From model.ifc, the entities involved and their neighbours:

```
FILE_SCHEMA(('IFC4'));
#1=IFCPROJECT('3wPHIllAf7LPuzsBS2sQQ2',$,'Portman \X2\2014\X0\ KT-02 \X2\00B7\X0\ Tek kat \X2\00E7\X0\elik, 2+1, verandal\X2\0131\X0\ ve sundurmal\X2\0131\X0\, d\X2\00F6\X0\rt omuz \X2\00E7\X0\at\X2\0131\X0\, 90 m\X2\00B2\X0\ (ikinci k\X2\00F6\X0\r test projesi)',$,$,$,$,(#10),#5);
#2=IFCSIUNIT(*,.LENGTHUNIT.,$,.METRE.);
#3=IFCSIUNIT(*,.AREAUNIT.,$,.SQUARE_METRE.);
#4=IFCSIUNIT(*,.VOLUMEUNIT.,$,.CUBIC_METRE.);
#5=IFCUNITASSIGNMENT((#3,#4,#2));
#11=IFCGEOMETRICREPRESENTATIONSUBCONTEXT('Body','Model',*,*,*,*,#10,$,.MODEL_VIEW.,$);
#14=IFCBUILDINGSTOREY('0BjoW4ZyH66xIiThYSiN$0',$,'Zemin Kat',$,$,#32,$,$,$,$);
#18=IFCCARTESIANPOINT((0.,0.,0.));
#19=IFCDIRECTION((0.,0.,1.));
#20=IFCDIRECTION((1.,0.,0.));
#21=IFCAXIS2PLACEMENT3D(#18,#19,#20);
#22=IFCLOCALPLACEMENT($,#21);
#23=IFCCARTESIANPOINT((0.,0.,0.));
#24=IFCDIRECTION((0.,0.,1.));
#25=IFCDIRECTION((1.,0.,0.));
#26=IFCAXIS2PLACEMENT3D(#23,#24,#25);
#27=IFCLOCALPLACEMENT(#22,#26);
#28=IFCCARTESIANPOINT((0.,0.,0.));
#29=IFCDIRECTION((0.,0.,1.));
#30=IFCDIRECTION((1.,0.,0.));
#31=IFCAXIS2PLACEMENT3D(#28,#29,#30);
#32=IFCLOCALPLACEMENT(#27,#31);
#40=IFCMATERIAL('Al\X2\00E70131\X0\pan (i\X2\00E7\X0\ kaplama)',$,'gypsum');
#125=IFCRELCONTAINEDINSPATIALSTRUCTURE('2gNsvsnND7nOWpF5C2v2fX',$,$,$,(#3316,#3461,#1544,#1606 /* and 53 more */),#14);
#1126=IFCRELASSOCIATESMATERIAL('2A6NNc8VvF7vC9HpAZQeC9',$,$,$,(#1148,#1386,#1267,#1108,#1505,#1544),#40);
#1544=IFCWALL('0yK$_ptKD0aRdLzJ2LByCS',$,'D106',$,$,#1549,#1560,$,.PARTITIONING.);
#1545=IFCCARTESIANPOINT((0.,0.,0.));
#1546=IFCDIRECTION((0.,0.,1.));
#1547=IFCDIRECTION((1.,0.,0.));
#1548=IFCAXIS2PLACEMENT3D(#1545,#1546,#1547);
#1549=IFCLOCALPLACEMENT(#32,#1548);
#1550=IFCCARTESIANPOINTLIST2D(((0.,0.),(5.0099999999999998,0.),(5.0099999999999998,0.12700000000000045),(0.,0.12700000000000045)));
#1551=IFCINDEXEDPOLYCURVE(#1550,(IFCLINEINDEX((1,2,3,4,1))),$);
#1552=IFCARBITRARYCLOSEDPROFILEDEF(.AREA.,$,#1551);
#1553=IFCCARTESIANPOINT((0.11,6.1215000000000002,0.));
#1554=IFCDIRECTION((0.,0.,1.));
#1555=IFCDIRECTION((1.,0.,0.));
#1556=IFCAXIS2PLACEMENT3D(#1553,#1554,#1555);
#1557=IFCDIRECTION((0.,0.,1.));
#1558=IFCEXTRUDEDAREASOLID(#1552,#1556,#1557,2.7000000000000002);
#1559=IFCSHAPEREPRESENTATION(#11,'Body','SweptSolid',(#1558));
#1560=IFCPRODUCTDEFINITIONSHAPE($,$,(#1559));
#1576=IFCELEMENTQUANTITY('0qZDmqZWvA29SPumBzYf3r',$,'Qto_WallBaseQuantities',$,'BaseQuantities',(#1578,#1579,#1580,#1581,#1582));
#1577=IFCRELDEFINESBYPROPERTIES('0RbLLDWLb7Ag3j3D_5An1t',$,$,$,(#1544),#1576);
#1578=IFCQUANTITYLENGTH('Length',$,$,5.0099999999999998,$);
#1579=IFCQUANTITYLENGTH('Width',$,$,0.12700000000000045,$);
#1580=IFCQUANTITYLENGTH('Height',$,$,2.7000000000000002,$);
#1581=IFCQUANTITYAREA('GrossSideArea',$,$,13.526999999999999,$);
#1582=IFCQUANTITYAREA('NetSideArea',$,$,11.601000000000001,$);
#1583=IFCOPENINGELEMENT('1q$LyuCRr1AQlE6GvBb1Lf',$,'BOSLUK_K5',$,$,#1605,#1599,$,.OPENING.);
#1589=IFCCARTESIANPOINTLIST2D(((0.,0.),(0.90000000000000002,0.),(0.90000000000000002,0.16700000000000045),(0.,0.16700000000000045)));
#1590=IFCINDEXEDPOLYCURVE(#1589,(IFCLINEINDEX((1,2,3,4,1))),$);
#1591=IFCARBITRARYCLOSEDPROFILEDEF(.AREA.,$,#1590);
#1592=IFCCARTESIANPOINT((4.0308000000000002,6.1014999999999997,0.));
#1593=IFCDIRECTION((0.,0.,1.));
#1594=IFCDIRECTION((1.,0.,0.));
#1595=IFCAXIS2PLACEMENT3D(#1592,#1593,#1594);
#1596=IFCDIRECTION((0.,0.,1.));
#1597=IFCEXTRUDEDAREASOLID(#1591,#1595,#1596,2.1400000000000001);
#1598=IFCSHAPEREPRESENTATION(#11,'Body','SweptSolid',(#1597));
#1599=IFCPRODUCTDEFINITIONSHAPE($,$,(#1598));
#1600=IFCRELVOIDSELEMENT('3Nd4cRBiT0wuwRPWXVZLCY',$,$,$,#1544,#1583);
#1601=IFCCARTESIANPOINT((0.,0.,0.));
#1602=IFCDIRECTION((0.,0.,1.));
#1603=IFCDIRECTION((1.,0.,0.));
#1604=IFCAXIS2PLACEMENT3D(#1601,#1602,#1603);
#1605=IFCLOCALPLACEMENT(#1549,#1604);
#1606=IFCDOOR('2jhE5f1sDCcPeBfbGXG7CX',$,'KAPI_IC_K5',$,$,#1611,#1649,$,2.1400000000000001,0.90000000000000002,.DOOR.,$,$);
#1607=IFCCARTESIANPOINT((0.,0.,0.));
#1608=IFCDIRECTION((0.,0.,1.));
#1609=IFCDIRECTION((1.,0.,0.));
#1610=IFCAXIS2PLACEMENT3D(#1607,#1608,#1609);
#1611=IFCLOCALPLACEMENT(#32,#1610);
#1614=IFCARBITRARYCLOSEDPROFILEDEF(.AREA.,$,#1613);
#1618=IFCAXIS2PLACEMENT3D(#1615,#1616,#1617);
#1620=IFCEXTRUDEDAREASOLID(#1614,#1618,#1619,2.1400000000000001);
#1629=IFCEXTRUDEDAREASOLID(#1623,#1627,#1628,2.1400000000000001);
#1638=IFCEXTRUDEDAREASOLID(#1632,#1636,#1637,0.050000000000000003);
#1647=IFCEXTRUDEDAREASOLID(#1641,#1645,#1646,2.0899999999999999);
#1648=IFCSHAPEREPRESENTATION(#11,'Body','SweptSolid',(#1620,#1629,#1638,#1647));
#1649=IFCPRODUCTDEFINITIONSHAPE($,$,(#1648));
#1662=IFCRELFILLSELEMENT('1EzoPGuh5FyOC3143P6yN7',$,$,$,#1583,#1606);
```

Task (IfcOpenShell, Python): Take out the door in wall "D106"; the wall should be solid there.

```python
import ifcopenshell
import ifcopenshell.api.feature
import ifcopenshell.api.pset
import ifcopenshell.api.root
import ifcopenshell.geom
import ifcopenshell.util.element
import ifcopenshell.util.shape
import ifcopenshell.util.unit

model = ifcopenshell.open("model.ifc")
area_scale = ifcopenshell.util.unit.calculate_unit_scale(model, "AREAUNIT")
settings = ifcopenshell.geom.settings()


def volume(element):
    """Net volume in cubic metres, openings subtracted."""
    shape = ifcopenshell.geom.create_shape(settings, element)
    return ifcopenshell.util.shape.get_volume(shape.geometry)


door = model.by_guid("2jhE5f1sDCcPeBfbGXG7CX")
opening = door.FillsVoids[0].RelatingOpeningElement
wall = opening.VoidsElements[0].RelatingBuildingElement
before = volume(wall)

ifcopenshell.api.root.remove_product(model, product=door)
ifcopenshell.api.feature.remove_feature(model, feature=opening)

after = volume(wall)
thickness = 0.127  # wall thickness in metres

# Update the wall's stored quantities.
qto = model.by_id(ifcopenshell.util.element.get_pset(wall, "Qto_WallBaseQuantities", should_inherit=False)["id"])
ifcopenshell.api.pset.edit_qto(model, qto=qto, properties={"NetSideArea": after / thickness / area_scale})

print(f"wall volume {before:.3f} -> {after:.3f} m3")

model.write("model-out.ifc")
```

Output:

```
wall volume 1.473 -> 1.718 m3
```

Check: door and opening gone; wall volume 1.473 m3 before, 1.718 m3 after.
